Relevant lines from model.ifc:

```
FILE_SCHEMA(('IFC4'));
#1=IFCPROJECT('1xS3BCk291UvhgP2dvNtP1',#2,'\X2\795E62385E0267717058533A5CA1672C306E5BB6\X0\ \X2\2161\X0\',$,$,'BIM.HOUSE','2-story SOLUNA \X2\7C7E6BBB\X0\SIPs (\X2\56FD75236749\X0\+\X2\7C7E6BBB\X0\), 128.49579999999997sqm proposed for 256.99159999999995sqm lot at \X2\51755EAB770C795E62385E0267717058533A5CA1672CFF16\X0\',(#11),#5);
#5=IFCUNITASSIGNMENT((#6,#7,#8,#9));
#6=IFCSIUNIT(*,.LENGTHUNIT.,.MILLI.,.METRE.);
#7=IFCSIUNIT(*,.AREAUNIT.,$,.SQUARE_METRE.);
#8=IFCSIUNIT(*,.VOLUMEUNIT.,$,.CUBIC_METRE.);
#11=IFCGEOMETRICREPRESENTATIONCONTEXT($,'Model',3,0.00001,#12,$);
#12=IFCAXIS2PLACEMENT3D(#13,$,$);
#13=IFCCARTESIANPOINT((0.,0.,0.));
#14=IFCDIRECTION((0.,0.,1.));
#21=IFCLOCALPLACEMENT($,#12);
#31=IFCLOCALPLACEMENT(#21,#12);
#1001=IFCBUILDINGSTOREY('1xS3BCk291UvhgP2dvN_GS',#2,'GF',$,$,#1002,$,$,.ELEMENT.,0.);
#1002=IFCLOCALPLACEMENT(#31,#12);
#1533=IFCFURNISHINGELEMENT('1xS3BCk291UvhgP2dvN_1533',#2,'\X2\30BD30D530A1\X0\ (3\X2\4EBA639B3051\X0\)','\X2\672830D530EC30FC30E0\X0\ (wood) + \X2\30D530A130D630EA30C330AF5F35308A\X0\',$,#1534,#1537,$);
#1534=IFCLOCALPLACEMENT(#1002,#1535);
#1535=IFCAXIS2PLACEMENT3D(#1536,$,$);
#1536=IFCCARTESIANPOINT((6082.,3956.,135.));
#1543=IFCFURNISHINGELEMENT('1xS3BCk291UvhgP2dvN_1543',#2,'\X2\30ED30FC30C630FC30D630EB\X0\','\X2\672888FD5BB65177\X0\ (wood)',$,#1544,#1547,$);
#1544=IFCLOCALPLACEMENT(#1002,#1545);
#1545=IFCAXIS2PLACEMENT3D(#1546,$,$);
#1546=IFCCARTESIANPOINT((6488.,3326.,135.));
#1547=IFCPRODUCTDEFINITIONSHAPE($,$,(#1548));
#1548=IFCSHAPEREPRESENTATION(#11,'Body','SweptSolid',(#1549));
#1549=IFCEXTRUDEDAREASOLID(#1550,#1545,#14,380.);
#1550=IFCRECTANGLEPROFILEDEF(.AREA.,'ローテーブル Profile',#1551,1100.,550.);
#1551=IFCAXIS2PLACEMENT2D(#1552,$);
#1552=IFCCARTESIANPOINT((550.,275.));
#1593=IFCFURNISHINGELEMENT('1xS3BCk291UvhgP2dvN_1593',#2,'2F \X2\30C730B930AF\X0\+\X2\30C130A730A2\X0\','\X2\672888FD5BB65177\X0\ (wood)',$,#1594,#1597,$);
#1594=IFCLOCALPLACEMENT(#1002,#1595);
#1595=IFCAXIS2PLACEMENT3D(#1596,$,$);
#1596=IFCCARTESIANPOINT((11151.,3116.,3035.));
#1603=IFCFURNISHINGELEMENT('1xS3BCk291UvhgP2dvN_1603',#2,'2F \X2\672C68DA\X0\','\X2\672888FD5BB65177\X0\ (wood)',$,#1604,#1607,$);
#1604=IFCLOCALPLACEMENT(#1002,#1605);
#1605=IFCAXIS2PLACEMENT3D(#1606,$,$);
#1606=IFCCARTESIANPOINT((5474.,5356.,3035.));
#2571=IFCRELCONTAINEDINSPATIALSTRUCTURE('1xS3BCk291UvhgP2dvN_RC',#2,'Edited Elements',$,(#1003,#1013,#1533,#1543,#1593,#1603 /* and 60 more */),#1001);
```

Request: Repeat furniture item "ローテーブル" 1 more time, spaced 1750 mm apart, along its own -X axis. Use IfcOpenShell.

```python
import ifcopenshell
import ifcopenshell.api.geometry
import ifcopenshell.api.root
import ifcopenshell.util.element
import ifcopenshell.util.placement

model = ifcopenshell.open("model.ifc")


def reuse_history(source, copy):
    """copy_class also copies each property set's owner history, people and application; keep the originals."""
    for rel in copy.IsDefinedBy:
        if rel.is_a("IfcRelDefinesByProperties") and (history := rel.RelatingPropertyDefinition.OwnerHistory):
            rel.RelatingPropertyDefinition.OwnerHistory = source.OwnerHistory
            ifcopenshell.util.element.remove_deep2(model, history)


source = model.by_guid("1xS3BCk291UvhgP2dvN_1543")
base = ifcopenshell.util.placement.get_local_placement(source.ObjectPlacement)
step = -base[:3, 0] * 1750.0

for i in range(1, 2):
    copy = ifcopenshell.api.root.copy_class(model, product=source)
    copy.Representation = ifcopenshell.util.element.copy_deep(
        model, source.Representation, exclude=["IfcGeometricRepresentationContext", "IfcRepresentationMap"]
    )
    reuse_history(source, copy)
    matrix = base.copy()
    matrix[:3, 3] += i * step
    print("added at", matrix[:3, 3].round(3) + 0.0)
    ifcopenshell.api.geometry.edit_object_placement(model, product=copy, matrix=matrix, is_si=False)

model.write("model_v2.ifc")
```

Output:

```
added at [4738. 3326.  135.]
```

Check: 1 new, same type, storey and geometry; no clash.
